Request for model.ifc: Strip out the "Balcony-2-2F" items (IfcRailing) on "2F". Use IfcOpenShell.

First a look at what the model holds.

```python
import ifcopenshell
import ifcopenshell.util.element

model = ifcopenshell.open("model.ifc")
print(model.schema)
storey = next(s for s in model.by_type("IfcBuildingStorey") if s.Name == "2F")
railings = [e for e in ifcopenshell.util.element.get_decomposition(storey) if e.is_a("IfcRailing")]
seen = {}
for e in railings:
    element_type = ifcopenshell.util.element.get_type(e)
    name = element_type.Name if element_type not in (None, e) else None
    seen[name] = seen.get(name, 0) + 1
for name, count in sorted(seen.items(), key=str):
    print(count, "x", name)
```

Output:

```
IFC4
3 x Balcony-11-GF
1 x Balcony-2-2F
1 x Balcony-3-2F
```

```python
import ifcopenshell
import ifcopenshell.api.root
import ifcopenshell.util.element

model = ifcopenshell.open("model.ifc")

storey = next(s for s in model.by_type("IfcBuildingStorey") if s.Name == "2F")
railings = [e for e in ifcopenshell.util.element.get_decomposition(storey) if e.is_a("IfcRailing")]
targets = [e for e in railings if (t := ifcopenshell.util.element.get_type(e)) not in (None, e) and t.Name == "Balcony-2-2F"]

for e in targets:
    ifcopenshell.api.root.remove_product(model, product=e)
print(len(targets), "removed")

model.write("model_rev.ifc")
```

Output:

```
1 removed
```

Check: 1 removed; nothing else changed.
